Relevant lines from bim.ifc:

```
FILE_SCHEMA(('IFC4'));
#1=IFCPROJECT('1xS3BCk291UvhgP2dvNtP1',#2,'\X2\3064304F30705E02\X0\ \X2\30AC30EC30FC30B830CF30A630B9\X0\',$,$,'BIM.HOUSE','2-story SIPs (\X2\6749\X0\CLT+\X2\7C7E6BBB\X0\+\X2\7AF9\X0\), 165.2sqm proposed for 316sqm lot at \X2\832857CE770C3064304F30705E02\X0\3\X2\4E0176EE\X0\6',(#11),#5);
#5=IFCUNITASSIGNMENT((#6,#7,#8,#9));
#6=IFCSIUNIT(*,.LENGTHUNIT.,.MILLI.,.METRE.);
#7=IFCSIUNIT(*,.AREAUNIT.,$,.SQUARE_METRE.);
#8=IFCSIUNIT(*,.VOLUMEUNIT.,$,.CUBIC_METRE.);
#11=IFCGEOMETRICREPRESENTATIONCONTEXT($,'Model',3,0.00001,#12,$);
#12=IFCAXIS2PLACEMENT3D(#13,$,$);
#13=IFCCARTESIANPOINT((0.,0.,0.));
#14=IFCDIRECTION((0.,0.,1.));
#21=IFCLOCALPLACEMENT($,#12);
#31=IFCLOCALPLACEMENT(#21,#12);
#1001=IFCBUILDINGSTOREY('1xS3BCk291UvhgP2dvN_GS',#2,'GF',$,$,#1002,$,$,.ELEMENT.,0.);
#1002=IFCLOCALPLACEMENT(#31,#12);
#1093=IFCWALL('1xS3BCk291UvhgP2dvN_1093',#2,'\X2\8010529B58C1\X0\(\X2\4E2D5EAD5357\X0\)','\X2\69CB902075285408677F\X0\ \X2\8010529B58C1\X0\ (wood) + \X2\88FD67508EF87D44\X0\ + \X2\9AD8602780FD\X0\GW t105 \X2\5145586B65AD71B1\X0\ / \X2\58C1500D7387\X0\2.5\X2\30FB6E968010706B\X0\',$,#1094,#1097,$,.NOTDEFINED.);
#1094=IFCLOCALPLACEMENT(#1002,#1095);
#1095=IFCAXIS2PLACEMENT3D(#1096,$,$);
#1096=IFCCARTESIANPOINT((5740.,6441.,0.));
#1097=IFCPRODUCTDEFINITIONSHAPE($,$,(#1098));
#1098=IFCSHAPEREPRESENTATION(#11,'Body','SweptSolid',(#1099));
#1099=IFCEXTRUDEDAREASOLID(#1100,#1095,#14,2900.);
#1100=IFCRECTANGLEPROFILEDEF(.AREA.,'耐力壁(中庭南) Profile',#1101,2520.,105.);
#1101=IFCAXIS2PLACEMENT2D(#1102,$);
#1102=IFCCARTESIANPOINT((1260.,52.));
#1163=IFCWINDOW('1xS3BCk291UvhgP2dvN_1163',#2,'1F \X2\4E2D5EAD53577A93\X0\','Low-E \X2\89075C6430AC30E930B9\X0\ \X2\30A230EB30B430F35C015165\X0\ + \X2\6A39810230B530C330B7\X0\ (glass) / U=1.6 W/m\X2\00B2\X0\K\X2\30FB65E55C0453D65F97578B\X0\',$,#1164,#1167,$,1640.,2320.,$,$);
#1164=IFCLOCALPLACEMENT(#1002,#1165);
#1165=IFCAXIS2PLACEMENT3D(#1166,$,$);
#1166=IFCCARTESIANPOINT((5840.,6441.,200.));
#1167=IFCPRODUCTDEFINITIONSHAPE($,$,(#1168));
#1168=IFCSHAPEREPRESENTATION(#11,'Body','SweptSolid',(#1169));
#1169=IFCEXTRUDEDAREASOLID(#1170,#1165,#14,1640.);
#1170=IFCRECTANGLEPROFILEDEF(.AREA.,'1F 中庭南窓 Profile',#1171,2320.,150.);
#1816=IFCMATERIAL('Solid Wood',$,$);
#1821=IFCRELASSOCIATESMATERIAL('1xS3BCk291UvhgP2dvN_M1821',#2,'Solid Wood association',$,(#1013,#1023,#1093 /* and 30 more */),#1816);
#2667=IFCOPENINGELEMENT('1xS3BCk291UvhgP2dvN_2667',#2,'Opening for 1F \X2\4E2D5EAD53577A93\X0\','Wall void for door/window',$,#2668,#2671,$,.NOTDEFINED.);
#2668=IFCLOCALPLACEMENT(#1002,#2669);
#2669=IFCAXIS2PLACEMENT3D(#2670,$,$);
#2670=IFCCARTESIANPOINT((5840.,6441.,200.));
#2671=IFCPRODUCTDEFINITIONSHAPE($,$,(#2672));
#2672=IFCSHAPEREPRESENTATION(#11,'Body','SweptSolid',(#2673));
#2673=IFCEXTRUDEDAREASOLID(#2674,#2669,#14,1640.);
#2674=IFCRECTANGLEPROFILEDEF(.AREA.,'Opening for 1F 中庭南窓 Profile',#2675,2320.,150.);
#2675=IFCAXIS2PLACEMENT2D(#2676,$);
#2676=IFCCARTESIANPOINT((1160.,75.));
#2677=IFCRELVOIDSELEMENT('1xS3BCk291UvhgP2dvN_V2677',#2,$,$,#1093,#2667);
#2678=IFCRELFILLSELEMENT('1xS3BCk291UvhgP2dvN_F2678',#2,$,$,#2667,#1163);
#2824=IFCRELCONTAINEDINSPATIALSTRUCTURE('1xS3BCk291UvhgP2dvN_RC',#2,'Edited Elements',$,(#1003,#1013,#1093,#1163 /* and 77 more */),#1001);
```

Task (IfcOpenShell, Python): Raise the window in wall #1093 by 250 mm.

```python
import numpy as np
import ifcopenshell
import ifcopenshell.api.geometry
import ifcopenshell.util.placement
import ifcopenshell.util.unit

model = ifcopenshell.open("bim.ifc")
unit_scale = ifcopenshell.util.unit.calculate_unit_scale(model)

window = model.by_guid("1xS3BCk291UvhgP2dvN_1163")
opening = window.FillsVoids[0].RelatingOpeningElement
dz = 250.0

shift = np.array([0.0, 0.0, dz])
# The window is not placed relative to its opening, so move both.
for product in (opening, window):
    matrix = ifcopenshell.util.placement.get_local_placement(product.ObjectPlacement)
    matrix[:3, 3] += shift
    ifcopenshell.api.geometry.edit_object_placement(model, product=product, matrix=matrix, is_si=False)

print(f"moved by {dz * unit_scale:+.3f} m")

model.write("bim_v2.ifc")
```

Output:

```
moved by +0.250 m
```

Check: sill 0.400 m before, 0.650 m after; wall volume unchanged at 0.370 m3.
